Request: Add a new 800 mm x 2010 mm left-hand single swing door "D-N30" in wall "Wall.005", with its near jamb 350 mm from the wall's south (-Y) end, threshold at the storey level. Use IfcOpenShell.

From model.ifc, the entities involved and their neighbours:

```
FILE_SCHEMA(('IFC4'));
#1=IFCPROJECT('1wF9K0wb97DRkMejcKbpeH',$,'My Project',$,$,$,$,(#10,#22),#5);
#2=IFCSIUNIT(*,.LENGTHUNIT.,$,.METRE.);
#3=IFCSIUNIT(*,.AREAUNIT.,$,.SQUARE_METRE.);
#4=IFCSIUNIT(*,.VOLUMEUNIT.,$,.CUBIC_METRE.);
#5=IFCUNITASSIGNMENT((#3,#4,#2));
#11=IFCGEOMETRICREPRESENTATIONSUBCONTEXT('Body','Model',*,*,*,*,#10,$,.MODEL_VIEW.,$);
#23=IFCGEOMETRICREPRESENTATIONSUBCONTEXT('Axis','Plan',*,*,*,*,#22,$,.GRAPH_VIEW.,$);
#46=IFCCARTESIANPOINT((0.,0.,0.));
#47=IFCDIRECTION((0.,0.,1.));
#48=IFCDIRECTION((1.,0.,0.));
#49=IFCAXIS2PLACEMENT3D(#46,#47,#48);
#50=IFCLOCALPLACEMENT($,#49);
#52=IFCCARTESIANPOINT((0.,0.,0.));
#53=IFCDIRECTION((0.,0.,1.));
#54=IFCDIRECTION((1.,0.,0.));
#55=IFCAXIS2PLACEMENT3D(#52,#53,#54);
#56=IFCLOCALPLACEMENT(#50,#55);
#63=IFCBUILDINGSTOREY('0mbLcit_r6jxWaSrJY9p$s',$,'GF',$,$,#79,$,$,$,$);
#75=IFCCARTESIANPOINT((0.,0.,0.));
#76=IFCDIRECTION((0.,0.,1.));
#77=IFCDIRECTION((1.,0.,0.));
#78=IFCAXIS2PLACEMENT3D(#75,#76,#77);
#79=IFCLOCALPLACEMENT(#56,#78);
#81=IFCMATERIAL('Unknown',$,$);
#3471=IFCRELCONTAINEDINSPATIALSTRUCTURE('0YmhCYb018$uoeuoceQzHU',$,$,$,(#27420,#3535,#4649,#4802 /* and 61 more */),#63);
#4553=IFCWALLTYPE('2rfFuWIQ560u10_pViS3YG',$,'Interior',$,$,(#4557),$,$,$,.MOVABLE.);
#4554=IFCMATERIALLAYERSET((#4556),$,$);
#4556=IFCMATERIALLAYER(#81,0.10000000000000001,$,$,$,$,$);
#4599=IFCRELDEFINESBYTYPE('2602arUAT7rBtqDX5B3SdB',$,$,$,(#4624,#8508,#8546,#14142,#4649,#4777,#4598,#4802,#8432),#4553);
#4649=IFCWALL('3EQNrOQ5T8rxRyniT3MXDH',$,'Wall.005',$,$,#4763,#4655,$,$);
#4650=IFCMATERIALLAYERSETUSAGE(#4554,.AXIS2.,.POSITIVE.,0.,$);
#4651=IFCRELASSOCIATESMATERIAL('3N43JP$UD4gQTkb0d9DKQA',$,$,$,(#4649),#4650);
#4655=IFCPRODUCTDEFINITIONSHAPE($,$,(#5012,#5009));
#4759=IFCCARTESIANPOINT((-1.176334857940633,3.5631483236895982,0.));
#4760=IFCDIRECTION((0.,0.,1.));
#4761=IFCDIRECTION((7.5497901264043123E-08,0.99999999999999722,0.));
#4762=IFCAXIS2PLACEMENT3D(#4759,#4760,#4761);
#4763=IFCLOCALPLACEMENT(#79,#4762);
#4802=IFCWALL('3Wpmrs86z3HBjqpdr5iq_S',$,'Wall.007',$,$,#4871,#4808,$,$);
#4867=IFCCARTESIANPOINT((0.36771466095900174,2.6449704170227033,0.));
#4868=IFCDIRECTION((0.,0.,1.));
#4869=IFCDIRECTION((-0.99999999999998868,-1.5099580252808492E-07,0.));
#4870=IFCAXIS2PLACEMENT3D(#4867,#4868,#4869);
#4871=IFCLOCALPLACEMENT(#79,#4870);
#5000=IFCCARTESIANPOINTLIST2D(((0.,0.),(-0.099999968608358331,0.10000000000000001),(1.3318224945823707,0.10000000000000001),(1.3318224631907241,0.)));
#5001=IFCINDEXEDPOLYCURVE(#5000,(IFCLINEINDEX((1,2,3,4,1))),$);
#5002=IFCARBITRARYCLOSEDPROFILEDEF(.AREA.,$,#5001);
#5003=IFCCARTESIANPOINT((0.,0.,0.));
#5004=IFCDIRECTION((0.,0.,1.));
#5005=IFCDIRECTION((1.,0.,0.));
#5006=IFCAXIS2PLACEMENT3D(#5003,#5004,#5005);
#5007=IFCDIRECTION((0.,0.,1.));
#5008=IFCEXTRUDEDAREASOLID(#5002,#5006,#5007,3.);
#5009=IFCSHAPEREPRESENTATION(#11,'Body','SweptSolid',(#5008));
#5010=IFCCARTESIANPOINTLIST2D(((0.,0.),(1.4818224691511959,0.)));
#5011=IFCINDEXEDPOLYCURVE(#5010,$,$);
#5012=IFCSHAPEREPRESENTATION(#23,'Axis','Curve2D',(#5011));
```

```python
import numpy as np
import ifcopenshell
import ifcopenshell.api.feature
import ifcopenshell.api.geometry
import ifcopenshell.api.root
import ifcopenshell.api.spatial
import ifcopenshell.geom
import ifcopenshell.util.element
import ifcopenshell.util.placement
import ifcopenshell.util.representation
import ifcopenshell.util.shape
import ifcopenshell.util.unit

model = ifcopenshell.open("model.ifc")
unit_scale = ifcopenshell.util.unit.calculate_unit_scale(model)
settings = ifcopenshell.geom.settings()


def volume(element):
    """Net volume in cubic metres, openings subtracted."""
    shape = ifcopenshell.geom.create_shape(settings, element)
    return ifcopenshell.util.shape.get_volume(shape.geometry)


wall = model.by_guid("3EQNrOQ5T8rxRyniT3MXDH")
storey = ifcopenshell.util.element.get_container(wall, ifc_class="IfcBuildingStorey")
context = ifcopenshell.util.representation.get_context(model, "Model", "Body", "MODEL_VIEW")
before = volume(wall)

width, height, from_end, sill = 0.8, 2.01, 0.35, 0.0  # metres

# The wall runs along its own X axis, and the end named is its -X end.
wall_shape = ifcopenshell.geom.create_shape(settings, wall)
x, y, z = ifcopenshell.util.shape.get_vertices(wall_shape.geometry).T
start = x.min() + from_end
face, thickness = float(y.min()), float(y.max() - y.min())
wall_matrix = ifcopenshell.util.placement.get_local_placement(wall.ObjectPlacement)
level = ifcopenshell.util.placement.get_local_placement(storey.ObjectPlacement)[2, 3]


def in_wall(x, y):
    """Placement at x, y metres in the wall's axes, at sill height."""
    matrix = wall_matrix.copy()
    matrix[:, 3] = wall_matrix @ np.array([x / unit_scale, y / unit_scale, 0.0, 1.0])
    matrix[2, 3] = level + sill / unit_scale
    return matrix


# Opening: a box that overshoots both wall faces by 50 mm.
opening = ifcopenshell.api.root.create_entity(model, ifc_class="IfcOpeningElement", predefined_type="OPENING")
box = ifcopenshell.api.geometry.add_wall_representation(
    model, context=context, length=width, height=height, thickness=thickness + 0.1
)
ifcopenshell.api.geometry.assign_representation(model, product=opening, representation=box)
ifcopenshell.api.geometry.edit_object_placement(model, product=opening, matrix=in_wall(start, face - 0.05), is_si=False)
ifcopenshell.api.feature.add_feature(model, feature=opening, element=wall)

door = ifcopenshell.api.root.create_entity(model, ifc_class="IfcDoor", name="D-N30", predefined_type="DOOR")
door.OverallWidth, door.OverallHeight = width / unit_scale, height / unit_scale
door.OperationType = "SINGLE_SWING_LEFT"
body = ifcopenshell.api.geometry.add_door_representation(
    model,
    context=context,
    overall_width=door.OverallWidth,
    overall_height=door.OverallHeight,
    operation_type="SINGLE_SWING_LEFT",
    lining_properties={"LiningDepth": thickness / unit_scale, "ThresholdDepth": thickness / unit_scale},
)
ifcopenshell.api.geometry.assign_representation(model, product=door, representation=body)
ifcopenshell.api.spatial.assign_container(model, products=[door], relating_structure=storey)
ifcopenshell.api.feature.add_filling(model, opening=opening, element=door)

# The lining spans the wall, so the door starts at the wall face.
ifcopenshell.api.geometry.edit_object_placement(model, product=door, matrix=in_wall(start, face), is_si=False)

after = volume(wall)

print(f"wall volume {before:.3f} -> {after:.3f} m3")

model.write("model-out.ifc")
```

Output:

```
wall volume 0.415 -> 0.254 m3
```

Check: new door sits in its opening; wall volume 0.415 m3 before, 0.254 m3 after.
